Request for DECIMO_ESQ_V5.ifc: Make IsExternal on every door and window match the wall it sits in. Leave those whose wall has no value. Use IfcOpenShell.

First a look at what the model holds.

```python
import ifcopenshell
import ifcopenshell.util.element

model = ifcopenshell.open("DECIMO_ESQ_V5.ifc")
print(model.schema)
seen = {}
for e in model.by_type("IfcDoor") + model.by_type("IfcWindow"):
    if not e.FillsVoids:
        continue
    host = e.FillsVoids[0].RelatingOpeningElement.VoidsElements[0].RelatingBuildingElement
    own = ifcopenshell.util.element.get_pset(e, f"Pset_{e.is_a()[3:].removesuffix('StandardCase')}Common", "IsExternal")
    wall = ifcopenshell.util.element.get_pset(host, "Pset_WallCommon", "IsExternal")
    seen[e.is_a(), own, wall] = seen.get((e.is_a(), own, wall), 0) + 1
for (cls, own, wall), count in sorted(seen.items(), key=str):
    print(count, cls, "IsExternal:", own, "| host wall:", wall)
```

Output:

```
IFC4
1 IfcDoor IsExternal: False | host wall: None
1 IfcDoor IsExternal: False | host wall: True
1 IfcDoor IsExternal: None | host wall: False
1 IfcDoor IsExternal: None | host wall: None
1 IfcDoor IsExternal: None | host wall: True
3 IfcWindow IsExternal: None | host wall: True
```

```python
import ifcopenshell
import ifcopenshell.api.pset
import ifcopenshell.util.element

model = ifcopenshell.open("DECIMO_ESQ_V5.ifc")

count = 0
for ifc_class, pset_name in (("IfcDoor", "Pset_DoorCommon"), ("IfcWindow", "Pset_WindowCommon")):
    for e in model.by_type(ifc_class):
        if not e.FillsVoids:
            continue
        host = e.FillsVoids[0].RelatingOpeningElement.VoidsElements[0].RelatingBuildingElement
        external = ifcopenshell.util.element.get_pset(host, "Pset_WallCommon", "IsExternal")
        if external is None or ifcopenshell.util.element.get_pset(e, pset_name, "IsExternal") == external:
            continue
        pset = ifcopenshell.api.pset.add_pset(model, product=e, name=pset_name)
        ifcopenshell.api.pset.edit_pset(model, pset=pset, properties={"IsExternal": external})
        count += 1

print(count, "updated")

model.write("DECIMO_ESQ_V5_v2.ifc")
```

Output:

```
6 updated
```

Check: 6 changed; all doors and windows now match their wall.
